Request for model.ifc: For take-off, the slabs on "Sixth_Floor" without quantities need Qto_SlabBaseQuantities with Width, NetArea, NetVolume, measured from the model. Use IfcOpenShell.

First a look at what the model holds.

```python
import ifcopenshell
import ifcopenshell.util.element
import ifcopenshell.util.unit

model = ifcopenshell.open("model.ifc")
print(model.schema)
for unit_type in ("LENGTHUNIT", "AREAUNIT", "VOLUMEUNIT"):
    print(unit_type, ifcopenshell.util.unit.calculate_unit_scale(model, unit_type))
storey = next(s for s in model.by_type("IfcBuildingStorey") if s.Name == "Sixth_Floor")
slabs = [e for e in ifcopenshell.util.element.get_decomposition(storey) if e.is_a("IfcSlab")]
for e in sorted(slabs, key=lambda e: e.id()):
    print(e.id(), e.is_a(), e.Name, list(ifcopenshell.util.element.get_psets(e, qtos_only=True)), sep=" | ")
```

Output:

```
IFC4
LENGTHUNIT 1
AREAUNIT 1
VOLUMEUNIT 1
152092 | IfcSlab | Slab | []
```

```python
import ifcopenshell
import ifcopenshell.api.pset
import ifcopenshell.geom
import ifcopenshell.util.element
import ifcopenshell.util.shape
import ifcopenshell.util.unit

model = ifcopenshell.open("model.ifc")
unit_scale = ifcopenshell.util.unit.calculate_unit_scale(model)
area_scale = ifcopenshell.util.unit.calculate_unit_scale(model, "AREAUNIT")
volume_scale = ifcopenshell.util.unit.calculate_unit_scale(model, "VOLUMEUNIT")
settings = ifcopenshell.geom.settings()

storey = next(s for s in model.by_type("IfcBuildingStorey") if s.Name == "Sixth_Floor")
slabs = [e for e in ifcopenshell.util.element.get_decomposition(storey) if e.is_a("IfcSlab")]

for e in sorted(slabs, key=lambda e: e.id()):
    if ifcopenshell.util.element.get_psets(e, qtos_only=True, should_inherit=False):
        continue
    # Geometry comes back in metres, in the element's own axes.
    shape = ifcopenshell.geom.create_shape(settings, e)
    values = {
        "Width": ifcopenshell.util.shape.get_z(shape.geometry) / unit_scale,
        "NetArea": ifcopenshell.util.shape.get_footprint_area(shape.geometry) / area_scale,
        "NetVolume": ifcopenshell.util.shape.get_volume(shape.geometry) / volume_scale,
    }
    qto = ifcopenshell.api.pset.add_qto(model, product=e, name="Qto_SlabBaseQuantities")
    ifcopenshell.api.pset.edit_qto(model, qto=qto, properties=values)
    print(e.id(), {k: round(v, 3) for k, v in values.items()})

model.write("model_updated.ifc")
```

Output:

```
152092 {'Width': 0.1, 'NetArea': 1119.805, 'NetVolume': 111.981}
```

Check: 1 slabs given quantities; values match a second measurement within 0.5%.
